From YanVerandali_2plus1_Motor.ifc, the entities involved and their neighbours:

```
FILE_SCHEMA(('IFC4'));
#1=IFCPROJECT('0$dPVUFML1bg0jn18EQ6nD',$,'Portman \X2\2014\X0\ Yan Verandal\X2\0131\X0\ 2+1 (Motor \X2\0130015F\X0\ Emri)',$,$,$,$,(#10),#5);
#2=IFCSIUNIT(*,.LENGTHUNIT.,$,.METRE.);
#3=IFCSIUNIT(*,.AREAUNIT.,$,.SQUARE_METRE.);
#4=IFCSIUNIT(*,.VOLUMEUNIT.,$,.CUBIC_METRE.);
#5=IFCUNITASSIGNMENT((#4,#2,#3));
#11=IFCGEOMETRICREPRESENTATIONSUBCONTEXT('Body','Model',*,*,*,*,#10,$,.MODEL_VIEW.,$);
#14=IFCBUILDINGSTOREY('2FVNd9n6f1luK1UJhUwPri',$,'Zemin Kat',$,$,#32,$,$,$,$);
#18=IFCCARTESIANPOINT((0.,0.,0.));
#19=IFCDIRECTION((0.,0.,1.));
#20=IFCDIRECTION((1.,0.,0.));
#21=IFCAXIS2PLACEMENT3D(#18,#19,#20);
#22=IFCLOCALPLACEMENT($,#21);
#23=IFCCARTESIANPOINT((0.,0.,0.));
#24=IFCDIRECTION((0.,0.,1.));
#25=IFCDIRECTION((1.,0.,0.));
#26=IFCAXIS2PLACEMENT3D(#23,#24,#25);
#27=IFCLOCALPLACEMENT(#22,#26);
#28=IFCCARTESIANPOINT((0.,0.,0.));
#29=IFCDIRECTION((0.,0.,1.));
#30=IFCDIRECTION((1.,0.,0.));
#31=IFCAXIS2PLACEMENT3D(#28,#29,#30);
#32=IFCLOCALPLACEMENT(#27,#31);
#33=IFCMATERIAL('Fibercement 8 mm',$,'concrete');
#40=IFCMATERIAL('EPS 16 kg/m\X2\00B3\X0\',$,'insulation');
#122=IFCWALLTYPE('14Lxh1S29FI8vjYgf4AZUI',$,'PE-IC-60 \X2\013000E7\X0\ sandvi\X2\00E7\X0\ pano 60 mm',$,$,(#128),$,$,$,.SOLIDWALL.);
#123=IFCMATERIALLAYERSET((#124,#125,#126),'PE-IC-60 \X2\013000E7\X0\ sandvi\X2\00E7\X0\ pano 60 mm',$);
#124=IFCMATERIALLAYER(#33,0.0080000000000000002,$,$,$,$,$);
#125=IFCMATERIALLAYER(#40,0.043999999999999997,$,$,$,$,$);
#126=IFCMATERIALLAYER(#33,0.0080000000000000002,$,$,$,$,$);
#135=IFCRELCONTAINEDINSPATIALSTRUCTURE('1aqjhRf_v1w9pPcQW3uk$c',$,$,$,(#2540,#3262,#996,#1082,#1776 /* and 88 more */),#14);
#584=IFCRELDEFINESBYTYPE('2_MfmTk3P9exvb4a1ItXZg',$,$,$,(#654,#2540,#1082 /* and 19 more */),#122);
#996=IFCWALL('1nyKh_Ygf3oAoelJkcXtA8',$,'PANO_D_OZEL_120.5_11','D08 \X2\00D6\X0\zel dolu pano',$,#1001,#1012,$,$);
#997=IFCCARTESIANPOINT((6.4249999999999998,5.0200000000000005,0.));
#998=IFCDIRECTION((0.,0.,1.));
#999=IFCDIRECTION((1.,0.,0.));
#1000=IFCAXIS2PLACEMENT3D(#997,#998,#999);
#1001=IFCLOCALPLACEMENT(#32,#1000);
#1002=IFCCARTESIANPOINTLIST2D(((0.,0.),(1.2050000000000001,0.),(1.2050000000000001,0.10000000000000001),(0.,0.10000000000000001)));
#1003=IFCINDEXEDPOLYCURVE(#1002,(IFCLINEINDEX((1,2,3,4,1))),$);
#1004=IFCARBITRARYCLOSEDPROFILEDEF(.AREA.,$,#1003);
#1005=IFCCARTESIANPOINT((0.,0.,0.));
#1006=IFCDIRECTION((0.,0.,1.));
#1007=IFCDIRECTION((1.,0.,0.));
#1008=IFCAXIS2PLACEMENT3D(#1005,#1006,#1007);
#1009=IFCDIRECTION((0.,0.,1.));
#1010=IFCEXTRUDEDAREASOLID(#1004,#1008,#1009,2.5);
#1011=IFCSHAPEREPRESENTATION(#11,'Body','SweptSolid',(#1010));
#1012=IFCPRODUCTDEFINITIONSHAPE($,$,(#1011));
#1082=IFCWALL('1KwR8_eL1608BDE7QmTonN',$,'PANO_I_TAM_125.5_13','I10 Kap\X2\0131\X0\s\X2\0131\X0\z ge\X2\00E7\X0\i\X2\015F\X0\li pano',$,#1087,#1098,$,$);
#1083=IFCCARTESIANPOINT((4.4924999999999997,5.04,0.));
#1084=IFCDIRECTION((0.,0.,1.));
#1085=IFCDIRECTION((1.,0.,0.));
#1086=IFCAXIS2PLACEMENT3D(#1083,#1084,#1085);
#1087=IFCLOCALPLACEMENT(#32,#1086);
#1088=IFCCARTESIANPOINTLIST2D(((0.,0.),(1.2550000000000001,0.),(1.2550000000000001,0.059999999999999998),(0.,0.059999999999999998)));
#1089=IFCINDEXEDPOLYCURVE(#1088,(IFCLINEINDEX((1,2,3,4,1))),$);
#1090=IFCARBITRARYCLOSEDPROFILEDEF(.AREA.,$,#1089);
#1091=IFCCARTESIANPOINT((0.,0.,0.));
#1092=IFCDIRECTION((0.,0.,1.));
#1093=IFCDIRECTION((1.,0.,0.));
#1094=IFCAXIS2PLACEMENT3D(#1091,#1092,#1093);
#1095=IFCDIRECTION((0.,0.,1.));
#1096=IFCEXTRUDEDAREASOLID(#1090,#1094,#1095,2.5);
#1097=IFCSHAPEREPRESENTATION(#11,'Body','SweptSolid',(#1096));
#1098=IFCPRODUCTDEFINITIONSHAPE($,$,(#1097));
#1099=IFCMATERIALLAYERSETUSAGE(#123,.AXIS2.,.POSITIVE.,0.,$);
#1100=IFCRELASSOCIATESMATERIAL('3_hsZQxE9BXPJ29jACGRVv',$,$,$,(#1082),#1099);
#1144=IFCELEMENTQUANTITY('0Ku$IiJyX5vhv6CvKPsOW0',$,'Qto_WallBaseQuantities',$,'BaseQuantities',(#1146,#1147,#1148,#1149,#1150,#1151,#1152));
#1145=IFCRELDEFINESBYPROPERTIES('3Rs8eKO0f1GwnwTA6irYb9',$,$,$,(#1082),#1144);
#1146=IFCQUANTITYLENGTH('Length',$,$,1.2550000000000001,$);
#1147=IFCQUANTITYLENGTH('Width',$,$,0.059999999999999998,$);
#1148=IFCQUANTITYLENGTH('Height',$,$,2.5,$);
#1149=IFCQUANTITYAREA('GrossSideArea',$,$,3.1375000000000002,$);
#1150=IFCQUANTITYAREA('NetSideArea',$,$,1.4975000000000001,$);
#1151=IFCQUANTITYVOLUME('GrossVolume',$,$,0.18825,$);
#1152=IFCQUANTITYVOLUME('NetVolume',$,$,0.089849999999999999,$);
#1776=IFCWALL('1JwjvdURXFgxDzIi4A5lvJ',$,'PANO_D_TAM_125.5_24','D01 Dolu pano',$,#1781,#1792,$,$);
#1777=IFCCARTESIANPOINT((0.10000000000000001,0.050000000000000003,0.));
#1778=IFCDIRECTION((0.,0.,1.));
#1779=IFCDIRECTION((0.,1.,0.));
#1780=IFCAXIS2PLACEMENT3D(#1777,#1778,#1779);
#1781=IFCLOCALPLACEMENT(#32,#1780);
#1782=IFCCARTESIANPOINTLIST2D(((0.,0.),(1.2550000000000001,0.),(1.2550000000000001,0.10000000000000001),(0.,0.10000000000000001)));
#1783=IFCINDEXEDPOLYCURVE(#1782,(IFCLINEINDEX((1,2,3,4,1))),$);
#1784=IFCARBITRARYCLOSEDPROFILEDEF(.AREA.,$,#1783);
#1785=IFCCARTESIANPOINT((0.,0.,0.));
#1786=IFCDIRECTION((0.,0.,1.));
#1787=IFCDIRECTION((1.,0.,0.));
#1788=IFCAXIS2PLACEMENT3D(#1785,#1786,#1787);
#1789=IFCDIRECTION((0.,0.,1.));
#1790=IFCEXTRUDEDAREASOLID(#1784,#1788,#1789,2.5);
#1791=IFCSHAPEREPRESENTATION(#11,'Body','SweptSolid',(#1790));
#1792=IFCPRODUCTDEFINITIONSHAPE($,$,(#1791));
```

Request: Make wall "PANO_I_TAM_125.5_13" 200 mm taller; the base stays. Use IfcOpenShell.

```python
import ifcopenshell
import ifcopenshell.api.pset
import ifcopenshell.geom
import ifcopenshell.util.element
import ifcopenshell.util.representation
import ifcopenshell.util.shape
import ifcopenshell.util.unit

model = ifcopenshell.open("YanVerandali_2plus1_Motor.ifc")
unit_scale = ifcopenshell.util.unit.calculate_unit_scale(model)
area_scale = ifcopenshell.util.unit.calculate_unit_scale(model, "AREAUNIT")
volume_scale = ifcopenshell.util.unit.calculate_unit_scale(model, "VOLUMEUNIT")
settings = ifcopenshell.geom.settings()


def volume(element):
    """Net volume in cubic metres, openings subtracted."""
    shape = ifcopenshell.geom.create_shape(settings, element)
    return ifcopenshell.util.shape.get_volume(shape.geometry)


wall = model.by_guid("1KwR8_eL1608BDE7QmTonN")
before = volume(wall)

body = ifcopenshell.util.representation.get_representation(wall, "Model", "Body")
solid = body.Items[0]
old_height = solid.Depth
solid.Depth += 0.2
after = volume(wall)
thickness = 0.06  # wall thickness in metres

# Update the stored height, areas and volumes.
qto = model.by_id(ifcopenshell.util.element.get_pset(wall, "Qto_WallBaseQuantities", should_inherit=False)["id"])
ifcopenshell.api.pset.edit_qto(model, qto=qto, properties={
    "Height": solid.Depth,
    "GrossSideArea": ifcopenshell.util.element.get_pset(wall, "Qto_WallBaseQuantities", "GrossSideArea") * solid.Depth / old_height,
    "NetSideArea": after / thickness / area_scale,
    "GrossVolume": ifcopenshell.util.element.get_pset(wall, "Qto_WallBaseQuantities", "GrossVolume") * solid.Depth / old_height,
    "NetVolume": after / volume_scale,
})

print(f"height {old_height:g} -> {solid.Depth:g}, volume {before:.3f} -> {after:.3f} m3")

model.write("YanVerandali_2plus1_Motor_edited.ifc")
```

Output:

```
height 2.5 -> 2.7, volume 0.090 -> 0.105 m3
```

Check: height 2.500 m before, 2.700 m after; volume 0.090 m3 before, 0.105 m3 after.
